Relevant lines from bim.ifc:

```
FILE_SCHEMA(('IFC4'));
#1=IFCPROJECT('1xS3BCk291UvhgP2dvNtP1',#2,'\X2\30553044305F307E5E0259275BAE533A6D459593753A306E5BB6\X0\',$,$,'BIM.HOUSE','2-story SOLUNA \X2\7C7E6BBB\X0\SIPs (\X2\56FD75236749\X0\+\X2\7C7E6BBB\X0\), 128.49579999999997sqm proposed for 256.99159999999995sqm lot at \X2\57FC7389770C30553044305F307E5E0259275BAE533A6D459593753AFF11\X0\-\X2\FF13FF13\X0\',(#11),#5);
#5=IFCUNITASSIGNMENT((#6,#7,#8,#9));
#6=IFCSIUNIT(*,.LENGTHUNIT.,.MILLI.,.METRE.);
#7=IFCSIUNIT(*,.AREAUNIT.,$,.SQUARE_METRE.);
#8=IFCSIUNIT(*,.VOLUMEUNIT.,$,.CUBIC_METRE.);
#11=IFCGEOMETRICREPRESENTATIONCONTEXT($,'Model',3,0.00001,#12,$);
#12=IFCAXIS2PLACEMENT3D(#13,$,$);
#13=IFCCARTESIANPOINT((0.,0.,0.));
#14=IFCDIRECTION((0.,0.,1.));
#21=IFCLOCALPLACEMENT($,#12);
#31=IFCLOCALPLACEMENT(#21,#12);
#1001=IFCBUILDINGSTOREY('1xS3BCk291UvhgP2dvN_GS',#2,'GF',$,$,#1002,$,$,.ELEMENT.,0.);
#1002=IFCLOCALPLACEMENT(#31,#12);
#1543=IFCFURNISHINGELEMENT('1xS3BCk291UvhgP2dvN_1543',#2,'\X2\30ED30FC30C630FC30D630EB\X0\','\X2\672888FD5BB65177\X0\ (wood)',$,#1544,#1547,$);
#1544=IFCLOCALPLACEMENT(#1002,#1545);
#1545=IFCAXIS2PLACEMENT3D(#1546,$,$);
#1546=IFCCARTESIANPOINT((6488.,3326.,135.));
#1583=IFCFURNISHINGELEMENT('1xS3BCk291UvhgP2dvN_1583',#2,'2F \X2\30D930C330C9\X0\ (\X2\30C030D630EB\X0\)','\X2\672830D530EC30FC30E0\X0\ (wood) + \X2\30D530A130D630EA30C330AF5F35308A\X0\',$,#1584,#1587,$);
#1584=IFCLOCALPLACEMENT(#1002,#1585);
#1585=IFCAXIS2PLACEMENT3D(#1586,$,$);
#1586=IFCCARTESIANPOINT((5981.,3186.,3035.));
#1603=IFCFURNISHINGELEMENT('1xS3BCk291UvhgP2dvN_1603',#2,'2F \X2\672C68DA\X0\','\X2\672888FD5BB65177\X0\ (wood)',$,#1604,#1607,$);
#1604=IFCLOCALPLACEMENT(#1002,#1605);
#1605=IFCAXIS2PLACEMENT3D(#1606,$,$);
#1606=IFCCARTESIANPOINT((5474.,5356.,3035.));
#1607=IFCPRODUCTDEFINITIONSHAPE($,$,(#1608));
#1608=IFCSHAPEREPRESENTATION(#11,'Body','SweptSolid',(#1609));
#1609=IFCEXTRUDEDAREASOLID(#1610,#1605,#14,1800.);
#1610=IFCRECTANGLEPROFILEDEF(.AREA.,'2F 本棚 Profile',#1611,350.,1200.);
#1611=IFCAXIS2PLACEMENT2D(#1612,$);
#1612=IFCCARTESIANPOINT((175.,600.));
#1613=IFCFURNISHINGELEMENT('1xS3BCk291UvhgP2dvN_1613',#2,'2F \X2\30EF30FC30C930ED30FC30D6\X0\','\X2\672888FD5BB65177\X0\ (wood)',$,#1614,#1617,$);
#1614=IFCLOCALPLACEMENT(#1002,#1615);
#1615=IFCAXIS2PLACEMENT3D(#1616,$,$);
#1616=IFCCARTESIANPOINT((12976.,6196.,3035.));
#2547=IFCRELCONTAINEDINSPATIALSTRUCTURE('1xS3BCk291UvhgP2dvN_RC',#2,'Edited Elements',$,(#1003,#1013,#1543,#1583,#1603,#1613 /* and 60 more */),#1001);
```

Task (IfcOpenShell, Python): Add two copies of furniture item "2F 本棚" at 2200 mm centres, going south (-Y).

```python
import numpy as np
import ifcopenshell
import ifcopenshell.api.geometry
import ifcopenshell.api.root
import ifcopenshell.util.element
import ifcopenshell.util.placement

model = ifcopenshell.open("bim.ifc")


def reuse_history(source, copy):
    """copy_class also copies each property set's owner history, people and application; keep the originals."""
    for rel in copy.IsDefinedBy:
        if rel.is_a("IfcRelDefinesByProperties") and (history := rel.RelatingPropertyDefinition.OwnerHistory):
            rel.RelatingPropertyDefinition.OwnerHistory = source.OwnerHistory
            ifcopenshell.util.element.remove_deep2(model, history)


source = model.by_id(1603)
base = ifcopenshell.util.placement.get_local_placement(source.ObjectPlacement)
step = np.array([0.0, -1.0, 0.0]) * 2200.0

for i in range(1, 3):
    copy = ifcopenshell.api.root.copy_class(model, product=source)
    copy.Representation = ifcopenshell.util.element.copy_deep(
        model, source.Representation, exclude=["IfcGeometricRepresentationContext", "IfcRepresentationMap"]
    )
    reuse_history(source, copy)
    matrix = base.copy()
    matrix[:3, 3] += i * step
    print("added at", matrix[:3, 3].round(3) + 0.0)
    ifcopenshell.api.geometry.edit_object_placement(model, product=copy, matrix=matrix, is_si=False)

model.write("bim_rev.ifc")
```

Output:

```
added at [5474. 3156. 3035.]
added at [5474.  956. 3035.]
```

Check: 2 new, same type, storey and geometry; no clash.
